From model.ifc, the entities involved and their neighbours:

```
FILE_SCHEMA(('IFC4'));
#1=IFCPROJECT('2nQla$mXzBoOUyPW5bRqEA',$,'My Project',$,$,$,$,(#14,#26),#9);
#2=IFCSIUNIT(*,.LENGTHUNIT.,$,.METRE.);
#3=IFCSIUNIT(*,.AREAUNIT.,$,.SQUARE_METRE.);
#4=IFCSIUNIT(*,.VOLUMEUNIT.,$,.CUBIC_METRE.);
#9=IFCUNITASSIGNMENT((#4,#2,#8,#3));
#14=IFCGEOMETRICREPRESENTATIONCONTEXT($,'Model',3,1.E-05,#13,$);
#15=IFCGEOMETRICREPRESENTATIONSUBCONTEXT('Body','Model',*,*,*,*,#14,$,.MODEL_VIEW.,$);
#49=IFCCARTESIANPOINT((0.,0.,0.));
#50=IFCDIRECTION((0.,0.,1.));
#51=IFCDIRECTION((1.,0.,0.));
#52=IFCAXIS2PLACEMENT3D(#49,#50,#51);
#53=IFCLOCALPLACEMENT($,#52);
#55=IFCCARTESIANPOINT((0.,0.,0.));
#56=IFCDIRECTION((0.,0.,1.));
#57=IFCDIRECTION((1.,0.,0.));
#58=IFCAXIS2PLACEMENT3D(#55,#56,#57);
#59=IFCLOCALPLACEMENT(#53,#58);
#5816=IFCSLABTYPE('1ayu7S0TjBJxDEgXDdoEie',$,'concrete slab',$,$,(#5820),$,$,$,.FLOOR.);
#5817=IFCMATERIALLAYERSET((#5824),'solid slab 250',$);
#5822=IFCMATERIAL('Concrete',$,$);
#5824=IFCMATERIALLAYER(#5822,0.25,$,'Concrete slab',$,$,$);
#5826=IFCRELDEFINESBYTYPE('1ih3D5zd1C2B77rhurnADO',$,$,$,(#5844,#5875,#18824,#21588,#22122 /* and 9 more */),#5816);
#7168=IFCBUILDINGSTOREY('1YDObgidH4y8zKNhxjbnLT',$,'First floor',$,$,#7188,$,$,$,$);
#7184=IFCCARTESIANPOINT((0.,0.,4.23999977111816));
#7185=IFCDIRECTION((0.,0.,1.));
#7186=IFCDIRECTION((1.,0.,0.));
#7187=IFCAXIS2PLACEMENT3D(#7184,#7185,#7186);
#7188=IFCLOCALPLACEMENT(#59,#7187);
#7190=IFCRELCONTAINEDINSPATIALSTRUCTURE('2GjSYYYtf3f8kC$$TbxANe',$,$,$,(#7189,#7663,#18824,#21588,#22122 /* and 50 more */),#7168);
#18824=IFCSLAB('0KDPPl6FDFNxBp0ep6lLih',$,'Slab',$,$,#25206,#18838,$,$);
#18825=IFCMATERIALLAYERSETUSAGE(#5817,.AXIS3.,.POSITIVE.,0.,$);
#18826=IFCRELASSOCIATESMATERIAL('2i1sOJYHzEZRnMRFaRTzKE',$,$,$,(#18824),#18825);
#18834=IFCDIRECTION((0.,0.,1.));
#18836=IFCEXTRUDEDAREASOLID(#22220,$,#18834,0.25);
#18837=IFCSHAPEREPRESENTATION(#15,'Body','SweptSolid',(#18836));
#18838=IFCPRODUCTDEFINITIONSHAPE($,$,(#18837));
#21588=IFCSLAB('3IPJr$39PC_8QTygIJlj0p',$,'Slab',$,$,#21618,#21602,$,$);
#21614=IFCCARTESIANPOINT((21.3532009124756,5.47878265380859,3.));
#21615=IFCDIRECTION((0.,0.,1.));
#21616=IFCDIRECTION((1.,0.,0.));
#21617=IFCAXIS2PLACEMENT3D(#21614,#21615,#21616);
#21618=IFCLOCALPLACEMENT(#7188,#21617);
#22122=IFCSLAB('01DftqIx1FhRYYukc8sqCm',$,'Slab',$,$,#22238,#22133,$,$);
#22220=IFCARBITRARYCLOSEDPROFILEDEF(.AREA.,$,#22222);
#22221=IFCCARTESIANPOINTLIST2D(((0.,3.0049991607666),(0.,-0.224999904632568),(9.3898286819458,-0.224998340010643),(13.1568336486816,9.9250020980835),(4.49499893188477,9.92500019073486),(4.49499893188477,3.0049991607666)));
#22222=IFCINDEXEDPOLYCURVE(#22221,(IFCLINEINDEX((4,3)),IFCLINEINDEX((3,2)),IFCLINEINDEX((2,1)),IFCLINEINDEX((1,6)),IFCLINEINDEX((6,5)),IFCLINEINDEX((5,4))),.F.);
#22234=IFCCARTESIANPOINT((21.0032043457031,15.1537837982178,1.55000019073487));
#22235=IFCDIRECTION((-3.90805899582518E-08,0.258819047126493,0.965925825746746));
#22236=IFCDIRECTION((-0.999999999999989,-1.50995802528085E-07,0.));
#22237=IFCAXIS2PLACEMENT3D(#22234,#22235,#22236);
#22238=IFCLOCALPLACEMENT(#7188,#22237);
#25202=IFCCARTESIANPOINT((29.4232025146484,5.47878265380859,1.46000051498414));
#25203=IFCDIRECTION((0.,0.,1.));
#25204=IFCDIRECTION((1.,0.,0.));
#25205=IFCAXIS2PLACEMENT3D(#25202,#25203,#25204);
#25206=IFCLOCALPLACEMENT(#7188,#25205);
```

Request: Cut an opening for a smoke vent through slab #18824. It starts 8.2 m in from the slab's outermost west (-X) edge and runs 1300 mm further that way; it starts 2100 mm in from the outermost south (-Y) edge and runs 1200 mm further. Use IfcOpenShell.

```python
import numpy as np
import ifcopenshell
import ifcopenshell.api.feature
import ifcopenshell.api.geometry
import ifcopenshell.api.root
import ifcopenshell.geom
import ifcopenshell.util.placement
import ifcopenshell.util.representation
import ifcopenshell.util.shape
import ifcopenshell.util.unit

model = ifcopenshell.open("model.ifc")
unit_scale = ifcopenshell.util.unit.calculate_unit_scale(model)
settings = ifcopenshell.geom.settings()


def volume(element):
    """Net volume in cubic metres, openings subtracted."""
    shape = ifcopenshell.geom.create_shape(settings, element)
    return ifcopenshell.util.shape.get_volume(shape.geometry)


slab = model.by_guid("0KDPPl6FDFNxBp0ep6lLih")
before = volume(slab)

# Extent in the slab's own axes, in metres. The edges named are its -X and -Y sides.
slab_shape = ifcopenshell.geom.create_shape(settings, slab)
vertices = ifcopenshell.util.shape.get_vertices(slab_shape.geometry)
x_min, y_min, bottom = vertices.min(axis=0)
top = vertices[:, 2].max()

opening = ifcopenshell.api.root.create_entity(model, ifc_class="IfcOpeningElement", name="Smoke vent opening", predefined_type="OPENING")
context = ifcopenshell.util.representation.get_context(model, "Model", "Body", "MODEL_VIEW")
width, depth = 1.3, 1.2
outline = [(0.0, 0.0), (width, 0.0), (width, depth), (0.0, depth), (0.0, 0.0)]
# Overshoot both faces by 50 mm so the cut is clean.
shape = ifcopenshell.api.geometry.add_slab_representation(
    model, context=context, depth=top - bottom + 0.1, polyline=outline
)
ifcopenshell.api.geometry.assign_representation(model, product=opening, representation=shape)

matrix = ifcopenshell.util.placement.get_local_placement(slab.ObjectPlacement)
matrix[:, 3] = matrix @ np.append(np.array([x_min + 8.2, y_min + 2.1, bottom - 0.05]) / unit_scale, 1.0)
ifcopenshell.api.geometry.edit_object_placement(model, product=opening, matrix=matrix, is_si=False)
ifcopenshell.api.feature.add_feature(model, feature=opening, element=slab)

after = volume(slab)

print(f"slab volume {before:.3f} -> {after:.3f} m3")

model.write("model_rev.ifc")
```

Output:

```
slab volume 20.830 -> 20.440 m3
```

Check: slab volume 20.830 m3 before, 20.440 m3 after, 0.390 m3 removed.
